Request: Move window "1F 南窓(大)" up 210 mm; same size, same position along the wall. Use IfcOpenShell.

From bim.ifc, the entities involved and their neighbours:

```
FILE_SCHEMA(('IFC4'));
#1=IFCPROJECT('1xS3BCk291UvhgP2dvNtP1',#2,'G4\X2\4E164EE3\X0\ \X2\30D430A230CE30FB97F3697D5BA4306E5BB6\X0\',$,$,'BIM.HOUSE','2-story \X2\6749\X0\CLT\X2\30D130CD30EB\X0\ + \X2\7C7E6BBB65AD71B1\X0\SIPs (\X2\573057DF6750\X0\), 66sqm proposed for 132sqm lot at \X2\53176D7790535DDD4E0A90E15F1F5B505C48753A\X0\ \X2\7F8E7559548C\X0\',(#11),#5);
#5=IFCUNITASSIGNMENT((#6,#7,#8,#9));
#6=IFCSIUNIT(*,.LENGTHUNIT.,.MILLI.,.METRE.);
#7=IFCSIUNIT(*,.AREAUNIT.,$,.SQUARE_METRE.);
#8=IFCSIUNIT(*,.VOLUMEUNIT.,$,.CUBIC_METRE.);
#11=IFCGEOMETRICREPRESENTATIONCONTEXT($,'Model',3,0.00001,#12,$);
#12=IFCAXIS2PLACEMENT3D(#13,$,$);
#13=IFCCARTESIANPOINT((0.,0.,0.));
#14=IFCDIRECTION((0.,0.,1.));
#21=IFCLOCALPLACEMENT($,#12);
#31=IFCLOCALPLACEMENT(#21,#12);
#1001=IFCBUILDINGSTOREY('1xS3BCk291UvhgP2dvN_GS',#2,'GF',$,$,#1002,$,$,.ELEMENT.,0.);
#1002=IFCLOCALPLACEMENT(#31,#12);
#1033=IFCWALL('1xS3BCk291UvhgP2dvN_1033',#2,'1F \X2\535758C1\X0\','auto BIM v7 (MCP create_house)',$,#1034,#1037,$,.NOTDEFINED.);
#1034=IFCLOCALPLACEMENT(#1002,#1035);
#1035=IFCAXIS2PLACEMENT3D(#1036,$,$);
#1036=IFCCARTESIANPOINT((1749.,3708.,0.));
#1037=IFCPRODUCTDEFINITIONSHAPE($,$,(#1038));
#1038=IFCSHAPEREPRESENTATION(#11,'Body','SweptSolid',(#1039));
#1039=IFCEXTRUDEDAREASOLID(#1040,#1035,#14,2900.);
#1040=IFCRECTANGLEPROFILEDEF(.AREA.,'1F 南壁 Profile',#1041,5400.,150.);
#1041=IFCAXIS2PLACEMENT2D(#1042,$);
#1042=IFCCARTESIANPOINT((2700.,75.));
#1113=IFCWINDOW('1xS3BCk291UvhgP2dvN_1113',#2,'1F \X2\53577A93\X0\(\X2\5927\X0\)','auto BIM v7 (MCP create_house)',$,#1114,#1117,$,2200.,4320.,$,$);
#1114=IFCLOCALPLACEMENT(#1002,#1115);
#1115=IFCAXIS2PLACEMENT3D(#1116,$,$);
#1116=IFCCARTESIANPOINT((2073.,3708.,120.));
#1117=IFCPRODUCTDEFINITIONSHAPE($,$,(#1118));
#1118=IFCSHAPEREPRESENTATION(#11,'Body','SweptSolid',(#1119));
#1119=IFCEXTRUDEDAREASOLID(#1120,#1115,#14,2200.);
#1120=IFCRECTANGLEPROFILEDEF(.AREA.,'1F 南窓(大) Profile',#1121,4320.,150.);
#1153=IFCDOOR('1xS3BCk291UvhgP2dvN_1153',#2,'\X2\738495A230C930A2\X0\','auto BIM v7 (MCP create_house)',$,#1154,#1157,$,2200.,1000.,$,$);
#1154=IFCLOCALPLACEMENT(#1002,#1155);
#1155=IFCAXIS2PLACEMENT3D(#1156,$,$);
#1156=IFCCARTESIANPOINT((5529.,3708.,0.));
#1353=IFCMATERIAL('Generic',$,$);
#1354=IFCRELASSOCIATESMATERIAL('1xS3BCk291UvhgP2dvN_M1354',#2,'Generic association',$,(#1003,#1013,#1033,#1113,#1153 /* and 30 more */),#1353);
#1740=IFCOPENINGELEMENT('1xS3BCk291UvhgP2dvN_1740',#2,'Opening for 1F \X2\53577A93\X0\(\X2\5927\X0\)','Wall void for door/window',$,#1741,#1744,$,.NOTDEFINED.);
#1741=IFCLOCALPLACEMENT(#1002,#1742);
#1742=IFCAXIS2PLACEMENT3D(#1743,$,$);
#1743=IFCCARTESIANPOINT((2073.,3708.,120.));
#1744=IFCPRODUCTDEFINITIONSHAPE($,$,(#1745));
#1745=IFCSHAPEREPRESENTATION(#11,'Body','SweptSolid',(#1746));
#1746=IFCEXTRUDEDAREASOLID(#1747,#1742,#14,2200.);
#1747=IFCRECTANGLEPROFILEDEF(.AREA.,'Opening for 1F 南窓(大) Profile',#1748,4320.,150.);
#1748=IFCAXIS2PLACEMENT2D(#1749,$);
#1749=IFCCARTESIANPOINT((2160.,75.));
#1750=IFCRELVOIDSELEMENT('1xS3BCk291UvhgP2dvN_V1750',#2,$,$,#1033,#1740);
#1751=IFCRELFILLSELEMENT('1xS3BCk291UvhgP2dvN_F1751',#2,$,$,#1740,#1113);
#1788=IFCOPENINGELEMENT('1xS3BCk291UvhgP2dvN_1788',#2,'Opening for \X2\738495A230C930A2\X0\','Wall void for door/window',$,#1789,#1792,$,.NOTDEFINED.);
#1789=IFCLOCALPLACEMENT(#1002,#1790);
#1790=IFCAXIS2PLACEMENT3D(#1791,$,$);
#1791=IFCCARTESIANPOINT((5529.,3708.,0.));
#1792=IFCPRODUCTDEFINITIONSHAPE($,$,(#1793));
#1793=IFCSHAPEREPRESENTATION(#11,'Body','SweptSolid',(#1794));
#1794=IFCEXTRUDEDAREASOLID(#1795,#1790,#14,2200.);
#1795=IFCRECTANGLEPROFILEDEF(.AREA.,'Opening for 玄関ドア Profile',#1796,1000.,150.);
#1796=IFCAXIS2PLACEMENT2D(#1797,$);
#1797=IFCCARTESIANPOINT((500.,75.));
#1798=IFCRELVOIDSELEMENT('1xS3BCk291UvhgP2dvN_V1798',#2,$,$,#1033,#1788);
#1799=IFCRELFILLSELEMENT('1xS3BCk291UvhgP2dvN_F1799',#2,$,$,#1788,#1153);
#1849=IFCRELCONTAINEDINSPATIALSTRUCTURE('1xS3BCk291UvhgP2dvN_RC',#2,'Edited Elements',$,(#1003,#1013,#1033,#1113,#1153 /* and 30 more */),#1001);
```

```python
import numpy as np
import ifcopenshell
import ifcopenshell.api.geometry
import ifcopenshell.util.placement
import ifcopenshell.util.unit

model = ifcopenshell.open("bim.ifc")
unit_scale = ifcopenshell.util.unit.calculate_unit_scale(model)

window = model.by_guid("1xS3BCk291UvhgP2dvN_1113")
opening = window.FillsVoids[0].RelatingOpeningElement
dz = 0.21 / unit_scale

shift = np.array([0.0, 0.0, dz])
# The window is not placed relative to its opening, so move both.
for product in (opening, window):
    matrix = ifcopenshell.util.placement.get_local_placement(product.ObjectPlacement)
    matrix[:3, 3] += shift
    ifcopenshell.api.geometry.edit_object_placement(model, product=product, matrix=matrix, is_si=False)

print(f"moved by {dz * unit_scale:+.3f} m")

model.write("bim_rev.ifc")
```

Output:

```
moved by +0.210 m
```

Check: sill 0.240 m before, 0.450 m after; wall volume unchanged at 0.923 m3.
